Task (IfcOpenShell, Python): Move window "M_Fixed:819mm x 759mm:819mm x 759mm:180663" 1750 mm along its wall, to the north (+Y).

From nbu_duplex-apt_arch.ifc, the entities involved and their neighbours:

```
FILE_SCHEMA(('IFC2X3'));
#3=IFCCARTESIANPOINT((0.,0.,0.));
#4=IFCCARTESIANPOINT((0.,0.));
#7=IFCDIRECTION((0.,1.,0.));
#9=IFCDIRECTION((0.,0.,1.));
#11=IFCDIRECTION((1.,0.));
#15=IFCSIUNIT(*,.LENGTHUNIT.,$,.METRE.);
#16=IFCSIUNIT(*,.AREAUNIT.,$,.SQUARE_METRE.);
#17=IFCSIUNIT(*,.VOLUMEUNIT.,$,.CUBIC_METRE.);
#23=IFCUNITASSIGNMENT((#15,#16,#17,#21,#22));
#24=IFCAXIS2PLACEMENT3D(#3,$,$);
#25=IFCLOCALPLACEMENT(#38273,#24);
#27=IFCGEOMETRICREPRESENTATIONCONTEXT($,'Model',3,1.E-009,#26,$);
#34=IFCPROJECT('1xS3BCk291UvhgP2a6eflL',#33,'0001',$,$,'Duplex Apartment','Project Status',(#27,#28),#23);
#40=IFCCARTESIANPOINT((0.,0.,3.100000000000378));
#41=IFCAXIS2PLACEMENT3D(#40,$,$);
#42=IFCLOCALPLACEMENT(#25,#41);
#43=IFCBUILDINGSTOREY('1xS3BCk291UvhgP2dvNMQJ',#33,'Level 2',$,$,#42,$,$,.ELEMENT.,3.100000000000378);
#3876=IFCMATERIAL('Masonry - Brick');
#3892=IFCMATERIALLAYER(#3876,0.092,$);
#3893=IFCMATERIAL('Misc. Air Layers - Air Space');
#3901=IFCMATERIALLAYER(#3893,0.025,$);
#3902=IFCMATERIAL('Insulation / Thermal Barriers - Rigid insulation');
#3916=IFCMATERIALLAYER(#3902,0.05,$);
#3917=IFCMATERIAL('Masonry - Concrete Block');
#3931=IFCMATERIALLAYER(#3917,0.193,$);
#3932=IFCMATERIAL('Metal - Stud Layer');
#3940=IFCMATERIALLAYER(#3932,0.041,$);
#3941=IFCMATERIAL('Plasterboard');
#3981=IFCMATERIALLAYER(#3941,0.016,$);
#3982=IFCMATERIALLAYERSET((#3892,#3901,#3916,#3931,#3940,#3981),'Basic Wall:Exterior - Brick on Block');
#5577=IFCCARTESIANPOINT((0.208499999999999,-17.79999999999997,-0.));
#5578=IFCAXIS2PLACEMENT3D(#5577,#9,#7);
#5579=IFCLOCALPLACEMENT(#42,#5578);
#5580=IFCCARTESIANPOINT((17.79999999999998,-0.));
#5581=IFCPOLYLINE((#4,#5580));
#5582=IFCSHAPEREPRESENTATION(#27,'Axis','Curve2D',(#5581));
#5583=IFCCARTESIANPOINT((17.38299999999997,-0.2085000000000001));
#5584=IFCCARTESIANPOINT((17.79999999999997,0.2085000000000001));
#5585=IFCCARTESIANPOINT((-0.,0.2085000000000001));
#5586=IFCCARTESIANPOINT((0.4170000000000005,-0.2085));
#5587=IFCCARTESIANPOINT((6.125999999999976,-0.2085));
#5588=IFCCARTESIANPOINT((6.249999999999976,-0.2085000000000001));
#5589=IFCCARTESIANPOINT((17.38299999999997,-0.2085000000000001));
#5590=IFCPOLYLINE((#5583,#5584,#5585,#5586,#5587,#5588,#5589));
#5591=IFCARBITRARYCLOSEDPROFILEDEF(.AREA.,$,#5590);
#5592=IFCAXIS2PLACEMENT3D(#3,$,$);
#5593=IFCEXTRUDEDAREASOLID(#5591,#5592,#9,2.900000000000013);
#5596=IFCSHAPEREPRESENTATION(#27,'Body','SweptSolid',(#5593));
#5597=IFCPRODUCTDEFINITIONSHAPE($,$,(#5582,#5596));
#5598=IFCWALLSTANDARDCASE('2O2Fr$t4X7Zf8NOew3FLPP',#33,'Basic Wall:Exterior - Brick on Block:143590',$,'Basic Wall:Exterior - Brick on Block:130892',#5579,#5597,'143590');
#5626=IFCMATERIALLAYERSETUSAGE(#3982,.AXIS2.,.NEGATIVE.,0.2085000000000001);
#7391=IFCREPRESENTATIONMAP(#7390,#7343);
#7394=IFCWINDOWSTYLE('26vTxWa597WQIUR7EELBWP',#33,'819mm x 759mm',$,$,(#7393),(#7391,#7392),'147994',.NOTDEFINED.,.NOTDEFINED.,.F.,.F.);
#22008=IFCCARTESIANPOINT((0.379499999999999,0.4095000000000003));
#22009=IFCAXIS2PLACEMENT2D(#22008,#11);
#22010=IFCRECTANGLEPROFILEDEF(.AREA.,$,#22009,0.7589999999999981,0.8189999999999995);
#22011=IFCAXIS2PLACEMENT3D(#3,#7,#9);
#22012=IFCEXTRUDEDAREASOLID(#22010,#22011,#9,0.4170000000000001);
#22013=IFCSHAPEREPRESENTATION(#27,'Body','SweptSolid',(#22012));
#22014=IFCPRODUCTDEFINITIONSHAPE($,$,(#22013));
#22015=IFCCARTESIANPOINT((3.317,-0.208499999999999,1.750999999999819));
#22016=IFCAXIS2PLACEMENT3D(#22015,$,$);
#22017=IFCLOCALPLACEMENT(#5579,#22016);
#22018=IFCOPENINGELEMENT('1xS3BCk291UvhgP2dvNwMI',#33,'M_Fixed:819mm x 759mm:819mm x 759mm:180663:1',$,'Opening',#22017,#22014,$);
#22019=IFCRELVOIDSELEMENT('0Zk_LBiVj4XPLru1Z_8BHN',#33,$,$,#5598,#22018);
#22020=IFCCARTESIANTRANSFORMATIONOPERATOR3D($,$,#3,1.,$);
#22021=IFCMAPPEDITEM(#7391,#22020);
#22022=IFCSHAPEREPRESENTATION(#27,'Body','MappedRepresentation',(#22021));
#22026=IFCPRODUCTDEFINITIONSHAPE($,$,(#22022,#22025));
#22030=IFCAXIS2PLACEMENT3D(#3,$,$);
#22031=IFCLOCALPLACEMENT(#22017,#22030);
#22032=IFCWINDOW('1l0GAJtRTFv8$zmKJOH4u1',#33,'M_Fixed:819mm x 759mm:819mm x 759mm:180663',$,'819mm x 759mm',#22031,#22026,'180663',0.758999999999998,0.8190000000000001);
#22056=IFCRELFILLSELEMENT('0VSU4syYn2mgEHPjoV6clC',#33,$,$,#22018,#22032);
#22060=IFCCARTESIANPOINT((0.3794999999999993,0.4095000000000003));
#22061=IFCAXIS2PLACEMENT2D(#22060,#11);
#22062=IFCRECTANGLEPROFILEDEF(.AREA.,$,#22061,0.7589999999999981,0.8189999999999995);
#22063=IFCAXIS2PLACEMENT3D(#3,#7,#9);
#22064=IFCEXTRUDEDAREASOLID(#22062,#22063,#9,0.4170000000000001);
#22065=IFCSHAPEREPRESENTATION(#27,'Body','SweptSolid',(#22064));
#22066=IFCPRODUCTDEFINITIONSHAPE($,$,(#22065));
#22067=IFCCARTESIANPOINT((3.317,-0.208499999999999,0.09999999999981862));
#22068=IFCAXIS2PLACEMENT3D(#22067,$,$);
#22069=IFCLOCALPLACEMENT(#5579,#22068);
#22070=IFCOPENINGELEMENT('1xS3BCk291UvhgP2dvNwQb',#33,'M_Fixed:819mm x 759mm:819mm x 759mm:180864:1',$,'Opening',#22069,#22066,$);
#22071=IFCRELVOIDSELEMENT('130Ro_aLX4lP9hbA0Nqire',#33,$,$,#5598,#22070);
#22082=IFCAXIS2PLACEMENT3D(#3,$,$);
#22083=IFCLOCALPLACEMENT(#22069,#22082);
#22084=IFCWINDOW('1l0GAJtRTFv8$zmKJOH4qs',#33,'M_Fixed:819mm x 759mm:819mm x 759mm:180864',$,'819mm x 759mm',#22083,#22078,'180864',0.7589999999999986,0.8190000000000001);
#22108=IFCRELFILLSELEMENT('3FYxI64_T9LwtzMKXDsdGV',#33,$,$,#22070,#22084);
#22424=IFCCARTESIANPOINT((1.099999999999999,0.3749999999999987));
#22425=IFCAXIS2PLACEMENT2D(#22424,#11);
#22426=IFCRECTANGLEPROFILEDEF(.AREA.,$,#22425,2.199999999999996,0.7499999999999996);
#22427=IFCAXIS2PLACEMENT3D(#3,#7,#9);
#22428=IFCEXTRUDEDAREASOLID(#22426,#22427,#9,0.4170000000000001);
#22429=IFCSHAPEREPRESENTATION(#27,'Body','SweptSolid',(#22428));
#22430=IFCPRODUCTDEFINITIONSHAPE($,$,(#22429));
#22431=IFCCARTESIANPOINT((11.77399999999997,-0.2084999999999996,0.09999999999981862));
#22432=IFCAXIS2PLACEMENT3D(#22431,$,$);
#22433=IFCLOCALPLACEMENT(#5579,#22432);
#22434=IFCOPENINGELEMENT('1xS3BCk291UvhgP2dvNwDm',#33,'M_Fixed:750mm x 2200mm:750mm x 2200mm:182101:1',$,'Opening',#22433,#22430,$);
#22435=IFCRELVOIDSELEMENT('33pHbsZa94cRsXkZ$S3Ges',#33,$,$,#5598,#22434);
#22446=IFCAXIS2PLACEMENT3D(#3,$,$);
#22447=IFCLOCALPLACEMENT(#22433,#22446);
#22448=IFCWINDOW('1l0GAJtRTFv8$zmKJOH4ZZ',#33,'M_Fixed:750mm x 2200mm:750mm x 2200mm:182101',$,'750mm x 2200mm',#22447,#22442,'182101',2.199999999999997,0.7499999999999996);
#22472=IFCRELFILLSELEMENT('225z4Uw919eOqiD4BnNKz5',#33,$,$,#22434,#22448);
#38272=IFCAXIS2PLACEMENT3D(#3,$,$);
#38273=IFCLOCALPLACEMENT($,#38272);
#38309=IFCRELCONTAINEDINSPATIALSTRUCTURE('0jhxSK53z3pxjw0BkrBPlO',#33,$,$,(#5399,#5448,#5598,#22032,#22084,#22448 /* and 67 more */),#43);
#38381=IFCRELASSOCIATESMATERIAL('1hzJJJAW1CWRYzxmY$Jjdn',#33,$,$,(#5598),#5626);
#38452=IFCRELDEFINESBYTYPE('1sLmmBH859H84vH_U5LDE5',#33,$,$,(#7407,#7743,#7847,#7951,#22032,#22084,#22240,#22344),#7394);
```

```python
import ifcopenshell
import ifcopenshell.api.geometry
import ifcopenshell.util.placement
import ifcopenshell.util.unit

model = ifcopenshell.open("nbu_duplex-apt_arch.ifc")
unit_scale = ifcopenshell.util.unit.calculate_unit_scale(model)

window = model.by_id(22032)
opening = window.FillsVoids[0].RelatingOpeningElement
wall = opening.VoidsElements[0].RelatingBuildingElement

wall_matrix = ifcopenshell.util.placement.get_local_placement(wall.ObjectPlacement)
shift = wall_matrix[:3, 0] * 1.75 / unit_scale
before = ifcopenshell.util.placement.get_local_placement(window.ObjectPlacement)[:3, 3].copy()

# The window is placed relative to its opening, so it follows when the opening moves.
matrix = ifcopenshell.util.placement.get_local_placement(opening.ObjectPlacement)
matrix[:3, 3] += shift
ifcopenshell.api.geometry.edit_object_placement(
    model, product=opening, matrix=matrix, is_si=False, should_transform_children=True
)

after = ifcopenshell.util.placement.get_local_placement(window.ObjectPlacement)[:3, 3]
print("window moved by", (after - before).round(3) + 0.0)

model.write("nbu_duplex-apt_arch_rev.ifc")
```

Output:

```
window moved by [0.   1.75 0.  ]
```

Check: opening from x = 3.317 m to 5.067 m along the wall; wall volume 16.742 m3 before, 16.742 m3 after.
